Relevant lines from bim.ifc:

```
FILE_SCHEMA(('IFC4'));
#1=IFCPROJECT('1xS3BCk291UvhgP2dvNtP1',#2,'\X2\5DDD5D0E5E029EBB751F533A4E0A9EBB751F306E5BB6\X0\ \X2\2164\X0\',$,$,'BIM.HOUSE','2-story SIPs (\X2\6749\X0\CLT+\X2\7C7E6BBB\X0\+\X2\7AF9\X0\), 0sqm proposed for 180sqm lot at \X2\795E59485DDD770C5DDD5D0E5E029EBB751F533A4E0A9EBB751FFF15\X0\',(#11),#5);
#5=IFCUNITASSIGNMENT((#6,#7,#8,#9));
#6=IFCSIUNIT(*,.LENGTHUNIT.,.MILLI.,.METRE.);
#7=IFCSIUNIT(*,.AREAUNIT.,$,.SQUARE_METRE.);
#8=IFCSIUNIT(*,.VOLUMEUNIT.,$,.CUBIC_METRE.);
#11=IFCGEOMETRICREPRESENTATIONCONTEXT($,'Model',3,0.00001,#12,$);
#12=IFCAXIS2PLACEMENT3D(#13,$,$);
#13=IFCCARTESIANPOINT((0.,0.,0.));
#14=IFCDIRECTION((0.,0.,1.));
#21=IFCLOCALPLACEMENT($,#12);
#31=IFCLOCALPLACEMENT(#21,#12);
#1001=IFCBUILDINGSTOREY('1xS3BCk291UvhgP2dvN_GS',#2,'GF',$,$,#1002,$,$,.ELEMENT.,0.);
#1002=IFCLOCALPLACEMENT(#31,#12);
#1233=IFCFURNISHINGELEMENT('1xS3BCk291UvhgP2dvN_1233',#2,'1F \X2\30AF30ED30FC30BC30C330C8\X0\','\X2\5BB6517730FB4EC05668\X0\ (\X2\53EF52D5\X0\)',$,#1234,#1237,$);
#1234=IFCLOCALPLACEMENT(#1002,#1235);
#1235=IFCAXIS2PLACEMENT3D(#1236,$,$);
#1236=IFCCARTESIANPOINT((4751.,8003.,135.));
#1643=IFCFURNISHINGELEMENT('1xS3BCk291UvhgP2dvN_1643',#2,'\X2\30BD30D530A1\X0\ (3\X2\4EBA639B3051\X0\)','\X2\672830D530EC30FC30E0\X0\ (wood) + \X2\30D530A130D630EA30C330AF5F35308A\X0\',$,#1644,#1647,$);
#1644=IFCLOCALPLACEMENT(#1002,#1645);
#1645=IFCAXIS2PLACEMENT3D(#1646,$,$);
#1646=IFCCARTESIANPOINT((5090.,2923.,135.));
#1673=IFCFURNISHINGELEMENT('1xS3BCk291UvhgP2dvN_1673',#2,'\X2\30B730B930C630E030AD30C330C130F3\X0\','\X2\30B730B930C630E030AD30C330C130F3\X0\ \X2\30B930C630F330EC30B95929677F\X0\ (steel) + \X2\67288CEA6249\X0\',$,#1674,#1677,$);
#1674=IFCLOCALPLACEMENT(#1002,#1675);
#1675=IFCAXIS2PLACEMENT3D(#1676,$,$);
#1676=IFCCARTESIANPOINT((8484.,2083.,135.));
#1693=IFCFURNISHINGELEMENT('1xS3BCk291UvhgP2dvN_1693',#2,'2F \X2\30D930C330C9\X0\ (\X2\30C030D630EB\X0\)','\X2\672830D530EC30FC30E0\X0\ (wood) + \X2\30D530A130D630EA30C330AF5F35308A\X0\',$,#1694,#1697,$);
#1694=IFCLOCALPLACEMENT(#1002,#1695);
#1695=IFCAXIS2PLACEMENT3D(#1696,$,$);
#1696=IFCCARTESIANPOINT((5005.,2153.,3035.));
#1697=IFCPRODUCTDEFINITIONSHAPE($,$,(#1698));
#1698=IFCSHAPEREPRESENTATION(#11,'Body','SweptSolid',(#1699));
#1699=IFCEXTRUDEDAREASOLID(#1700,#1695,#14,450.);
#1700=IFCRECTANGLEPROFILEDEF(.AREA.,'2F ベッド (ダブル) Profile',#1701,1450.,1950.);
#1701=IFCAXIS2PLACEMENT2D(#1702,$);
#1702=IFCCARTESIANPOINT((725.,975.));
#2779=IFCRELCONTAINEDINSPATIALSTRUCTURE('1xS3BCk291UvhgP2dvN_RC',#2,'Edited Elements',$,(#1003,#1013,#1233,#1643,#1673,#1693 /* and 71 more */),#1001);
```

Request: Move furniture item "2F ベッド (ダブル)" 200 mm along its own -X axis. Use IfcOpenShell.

```python
import ifcopenshell
import ifcopenshell.api.geometry
import ifcopenshell.util.placement

model = ifcopenshell.open("bim.ifc")

item = model.by_guid("1xS3BCk291UvhgP2dvN_1693")
matrix = ifcopenshell.util.placement.get_local_placement(item.ObjectPlacement)
matrix[:3, 3] -= matrix[:3, 0] * 200.0
ifcopenshell.api.geometry.edit_object_placement(model, product=item, matrix=matrix, is_si=False)

print(ifcopenshell.util.placement.get_local_placement(item.ObjectPlacement).round(3) + 0.0)

model.write("bim_edited.ifc")
```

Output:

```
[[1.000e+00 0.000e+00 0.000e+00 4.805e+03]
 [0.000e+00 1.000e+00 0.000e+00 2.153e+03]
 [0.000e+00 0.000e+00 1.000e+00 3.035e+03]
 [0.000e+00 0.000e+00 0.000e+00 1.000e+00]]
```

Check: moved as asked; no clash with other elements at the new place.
